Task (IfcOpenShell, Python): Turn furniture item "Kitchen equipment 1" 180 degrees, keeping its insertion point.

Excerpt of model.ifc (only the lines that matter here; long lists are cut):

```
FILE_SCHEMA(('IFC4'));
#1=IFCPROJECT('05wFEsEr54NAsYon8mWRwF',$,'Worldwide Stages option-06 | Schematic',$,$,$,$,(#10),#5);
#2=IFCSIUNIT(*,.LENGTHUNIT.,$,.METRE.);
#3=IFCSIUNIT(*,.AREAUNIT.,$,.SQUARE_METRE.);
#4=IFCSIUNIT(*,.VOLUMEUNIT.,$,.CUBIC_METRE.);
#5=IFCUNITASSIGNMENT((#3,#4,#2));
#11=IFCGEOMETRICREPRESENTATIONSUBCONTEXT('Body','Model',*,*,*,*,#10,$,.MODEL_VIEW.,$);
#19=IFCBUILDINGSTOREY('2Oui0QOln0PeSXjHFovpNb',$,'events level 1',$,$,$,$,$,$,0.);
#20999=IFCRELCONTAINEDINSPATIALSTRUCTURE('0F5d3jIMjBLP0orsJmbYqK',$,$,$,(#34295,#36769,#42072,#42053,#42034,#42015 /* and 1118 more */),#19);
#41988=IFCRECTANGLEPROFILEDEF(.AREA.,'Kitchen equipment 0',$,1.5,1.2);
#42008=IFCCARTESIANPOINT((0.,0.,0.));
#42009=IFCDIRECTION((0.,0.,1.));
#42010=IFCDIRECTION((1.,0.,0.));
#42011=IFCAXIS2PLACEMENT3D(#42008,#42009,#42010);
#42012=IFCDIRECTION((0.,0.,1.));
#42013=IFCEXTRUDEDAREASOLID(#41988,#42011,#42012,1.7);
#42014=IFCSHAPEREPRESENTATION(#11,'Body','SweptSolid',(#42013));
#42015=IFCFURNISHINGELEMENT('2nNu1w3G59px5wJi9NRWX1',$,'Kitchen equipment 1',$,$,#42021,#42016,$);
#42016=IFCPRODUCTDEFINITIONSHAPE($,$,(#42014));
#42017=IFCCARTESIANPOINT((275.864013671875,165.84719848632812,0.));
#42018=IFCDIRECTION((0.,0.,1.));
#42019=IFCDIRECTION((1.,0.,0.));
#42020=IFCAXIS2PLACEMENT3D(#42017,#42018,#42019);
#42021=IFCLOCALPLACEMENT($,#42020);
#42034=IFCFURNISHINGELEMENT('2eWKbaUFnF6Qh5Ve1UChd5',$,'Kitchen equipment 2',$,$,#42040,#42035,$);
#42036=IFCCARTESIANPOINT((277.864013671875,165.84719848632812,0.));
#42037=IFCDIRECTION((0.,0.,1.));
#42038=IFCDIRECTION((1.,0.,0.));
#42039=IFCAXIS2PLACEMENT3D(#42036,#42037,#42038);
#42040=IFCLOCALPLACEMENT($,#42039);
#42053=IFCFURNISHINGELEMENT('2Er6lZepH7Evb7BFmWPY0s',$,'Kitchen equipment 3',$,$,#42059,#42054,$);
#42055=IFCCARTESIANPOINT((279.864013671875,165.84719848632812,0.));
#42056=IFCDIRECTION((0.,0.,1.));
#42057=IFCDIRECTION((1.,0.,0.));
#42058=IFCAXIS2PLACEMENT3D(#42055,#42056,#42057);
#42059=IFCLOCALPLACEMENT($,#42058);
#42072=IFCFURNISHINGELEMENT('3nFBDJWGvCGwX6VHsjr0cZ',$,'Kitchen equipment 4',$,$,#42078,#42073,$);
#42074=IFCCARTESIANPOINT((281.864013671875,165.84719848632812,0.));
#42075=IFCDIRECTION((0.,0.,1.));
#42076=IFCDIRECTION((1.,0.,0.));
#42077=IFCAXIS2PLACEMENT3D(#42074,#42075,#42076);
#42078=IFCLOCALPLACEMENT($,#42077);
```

```python
import ifcopenshell
import ifcopenshell.api.geometry
import ifcopenshell.util.placement

model = ifcopenshell.open("model.ifc")

item = model.by_id(42015)
matrix = ifcopenshell.util.placement.get_local_placement(item.ObjectPlacement)
matrix = matrix @ ifcopenshell.util.placement.rotation(180, "Z")
ifcopenshell.api.geometry.edit_object_placement(model, product=item, matrix=matrix, is_si=False)

print(ifcopenshell.util.placement.get_local_placement(item.ObjectPlacement).round(3) + 0.0)

model.write("model_updated.ifc")
```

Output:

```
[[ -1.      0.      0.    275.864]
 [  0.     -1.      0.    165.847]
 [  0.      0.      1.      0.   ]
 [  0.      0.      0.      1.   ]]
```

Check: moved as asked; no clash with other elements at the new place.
